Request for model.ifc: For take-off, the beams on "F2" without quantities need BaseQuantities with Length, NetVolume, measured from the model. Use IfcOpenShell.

First a look at what the model holds.

```python
import ifcopenshell
import ifcopenshell.util.element
import ifcopenshell.util.unit

model = ifcopenshell.open("model.ifc")
print(model.schema)
for unit_type in ("LENGTHUNIT", "AREAUNIT", "VOLUMEUNIT"):
    print(unit_type, ifcopenshell.util.unit.calculate_unit_scale(model, unit_type))
storey = next(s for s in model.by_type("IfcBuildingStorey") if s.Name == "F2")
beams = [e for e in ifcopenshell.util.element.get_decomposition(storey) if e.is_a("IfcBeam")]
for e in sorted(beams, key=lambda e: e.id()):
    print(e.id(), e.is_a(), e.Name, list(ifcopenshell.util.element.get_psets(e, qtos_only=True)), sep=" | ")
```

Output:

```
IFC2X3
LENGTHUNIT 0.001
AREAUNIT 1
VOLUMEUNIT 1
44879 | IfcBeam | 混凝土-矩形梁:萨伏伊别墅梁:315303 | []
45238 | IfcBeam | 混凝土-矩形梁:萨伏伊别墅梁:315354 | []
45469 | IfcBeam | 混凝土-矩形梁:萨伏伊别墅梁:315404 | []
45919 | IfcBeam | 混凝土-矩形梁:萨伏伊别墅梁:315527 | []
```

```python
import ifcopenshell
import ifcopenshell.api.pset
import ifcopenshell.geom
import ifcopenshell.util.element
import ifcopenshell.util.shape
import ifcopenshell.util.unit

model = ifcopenshell.open("model.ifc")
unit_scale = ifcopenshell.util.unit.calculate_unit_scale(model)
volume_scale = ifcopenshell.util.unit.calculate_unit_scale(model, "VOLUMEUNIT")
settings = ifcopenshell.geom.settings()

storey = next(s for s in model.by_type("IfcBuildingStorey") if s.Name == "F2")
beams = [e for e in ifcopenshell.util.element.get_decomposition(storey) if e.is_a("IfcBeam")]

for e in sorted(beams, key=lambda e: e.id()):
    if ifcopenshell.util.element.get_psets(e, qtos_only=True, should_inherit=False):
        continue
    # Geometry comes back in metres, in the element's own axes.
    shape = ifcopenshell.geom.create_shape(settings, e)
    values = {
        "Length": ifcopenshell.util.shape.get_max_xyz(shape.geometry) / unit_scale,
        "NetVolume": ifcopenshell.util.shape.get_volume(shape.geometry) / volume_scale,
    }
    qto = ifcopenshell.api.pset.add_qto(model, product=e, name="BaseQuantities")
    ifcopenshell.api.pset.edit_qto(model, qto=qto, properties=values)
    print(e.id(), {k: round(v, 3) for k, v in values.items()})

model.write("model_rev.ifc")
```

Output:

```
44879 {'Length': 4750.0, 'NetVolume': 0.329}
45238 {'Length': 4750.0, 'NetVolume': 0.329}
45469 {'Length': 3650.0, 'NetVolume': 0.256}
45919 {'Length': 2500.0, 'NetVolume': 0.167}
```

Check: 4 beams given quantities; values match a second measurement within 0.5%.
